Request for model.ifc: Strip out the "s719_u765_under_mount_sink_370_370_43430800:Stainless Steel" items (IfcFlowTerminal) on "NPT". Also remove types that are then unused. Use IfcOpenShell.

First a look at what the model holds.

```python
import ifcopenshell
import ifcopenshell.util.element

model = ifcopenshell.open("model.ifc")
print(model.schema)
storey = next(s for s in model.by_type("IfcBuildingStorey") if s.Name == "NPT")
terminals = [e for e in ifcopenshell.util.element.get_decomposition(storey) if e.is_a("IfcFlowTerminal")]
seen = {}
for e in terminals:
    element_type = ifcopenshell.util.element.get_type(e)
    name = element_type.Name if element_type not in (None, e) else None
    seen[name] = seen.get(name, 0) + 1
for name, count in sorted(seen.items(), key=str):
    print(count, "x", name)
```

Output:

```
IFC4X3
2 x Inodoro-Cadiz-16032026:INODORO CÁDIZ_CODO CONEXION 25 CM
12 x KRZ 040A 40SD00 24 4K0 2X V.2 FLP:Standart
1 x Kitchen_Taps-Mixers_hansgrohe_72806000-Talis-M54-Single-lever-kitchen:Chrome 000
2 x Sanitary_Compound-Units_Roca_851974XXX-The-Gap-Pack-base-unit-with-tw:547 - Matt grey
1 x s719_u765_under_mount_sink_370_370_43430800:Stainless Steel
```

```python
import ifcopenshell
import ifcopenshell.api.root
import ifcopenshell.util.element

model = ifcopenshell.open("model.ifc")

storey = next(s for s in model.by_type("IfcBuildingStorey") if s.Name == "NPT")
terminals = [e for e in ifcopenshell.util.element.get_decomposition(storey) if e.is_a("IfcFlowTerminal")]
targets = [e for e in terminals if (t := ifcopenshell.util.element.get_type(e)) not in (None, e) and t.Name == "s719_u765_under_mount_sink_370_370_43430800:Stainless Steel"]
types = {ifcopenshell.util.element.get_type(e) for e in targets} - {None, *targets}

for e in targets:
    ifcopenshell.api.root.remove_product(model, product=e)
print(len(targets), "removed")

unused = [t for t in types if not ifcopenshell.util.element.get_types(t)]
for t in unused:
    ifcopenshell.api.root.remove_product(model, product=t)
print(len(unused), "unused types removed")

model.write("model_updated.ifc")
```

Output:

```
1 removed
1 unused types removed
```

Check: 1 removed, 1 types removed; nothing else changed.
